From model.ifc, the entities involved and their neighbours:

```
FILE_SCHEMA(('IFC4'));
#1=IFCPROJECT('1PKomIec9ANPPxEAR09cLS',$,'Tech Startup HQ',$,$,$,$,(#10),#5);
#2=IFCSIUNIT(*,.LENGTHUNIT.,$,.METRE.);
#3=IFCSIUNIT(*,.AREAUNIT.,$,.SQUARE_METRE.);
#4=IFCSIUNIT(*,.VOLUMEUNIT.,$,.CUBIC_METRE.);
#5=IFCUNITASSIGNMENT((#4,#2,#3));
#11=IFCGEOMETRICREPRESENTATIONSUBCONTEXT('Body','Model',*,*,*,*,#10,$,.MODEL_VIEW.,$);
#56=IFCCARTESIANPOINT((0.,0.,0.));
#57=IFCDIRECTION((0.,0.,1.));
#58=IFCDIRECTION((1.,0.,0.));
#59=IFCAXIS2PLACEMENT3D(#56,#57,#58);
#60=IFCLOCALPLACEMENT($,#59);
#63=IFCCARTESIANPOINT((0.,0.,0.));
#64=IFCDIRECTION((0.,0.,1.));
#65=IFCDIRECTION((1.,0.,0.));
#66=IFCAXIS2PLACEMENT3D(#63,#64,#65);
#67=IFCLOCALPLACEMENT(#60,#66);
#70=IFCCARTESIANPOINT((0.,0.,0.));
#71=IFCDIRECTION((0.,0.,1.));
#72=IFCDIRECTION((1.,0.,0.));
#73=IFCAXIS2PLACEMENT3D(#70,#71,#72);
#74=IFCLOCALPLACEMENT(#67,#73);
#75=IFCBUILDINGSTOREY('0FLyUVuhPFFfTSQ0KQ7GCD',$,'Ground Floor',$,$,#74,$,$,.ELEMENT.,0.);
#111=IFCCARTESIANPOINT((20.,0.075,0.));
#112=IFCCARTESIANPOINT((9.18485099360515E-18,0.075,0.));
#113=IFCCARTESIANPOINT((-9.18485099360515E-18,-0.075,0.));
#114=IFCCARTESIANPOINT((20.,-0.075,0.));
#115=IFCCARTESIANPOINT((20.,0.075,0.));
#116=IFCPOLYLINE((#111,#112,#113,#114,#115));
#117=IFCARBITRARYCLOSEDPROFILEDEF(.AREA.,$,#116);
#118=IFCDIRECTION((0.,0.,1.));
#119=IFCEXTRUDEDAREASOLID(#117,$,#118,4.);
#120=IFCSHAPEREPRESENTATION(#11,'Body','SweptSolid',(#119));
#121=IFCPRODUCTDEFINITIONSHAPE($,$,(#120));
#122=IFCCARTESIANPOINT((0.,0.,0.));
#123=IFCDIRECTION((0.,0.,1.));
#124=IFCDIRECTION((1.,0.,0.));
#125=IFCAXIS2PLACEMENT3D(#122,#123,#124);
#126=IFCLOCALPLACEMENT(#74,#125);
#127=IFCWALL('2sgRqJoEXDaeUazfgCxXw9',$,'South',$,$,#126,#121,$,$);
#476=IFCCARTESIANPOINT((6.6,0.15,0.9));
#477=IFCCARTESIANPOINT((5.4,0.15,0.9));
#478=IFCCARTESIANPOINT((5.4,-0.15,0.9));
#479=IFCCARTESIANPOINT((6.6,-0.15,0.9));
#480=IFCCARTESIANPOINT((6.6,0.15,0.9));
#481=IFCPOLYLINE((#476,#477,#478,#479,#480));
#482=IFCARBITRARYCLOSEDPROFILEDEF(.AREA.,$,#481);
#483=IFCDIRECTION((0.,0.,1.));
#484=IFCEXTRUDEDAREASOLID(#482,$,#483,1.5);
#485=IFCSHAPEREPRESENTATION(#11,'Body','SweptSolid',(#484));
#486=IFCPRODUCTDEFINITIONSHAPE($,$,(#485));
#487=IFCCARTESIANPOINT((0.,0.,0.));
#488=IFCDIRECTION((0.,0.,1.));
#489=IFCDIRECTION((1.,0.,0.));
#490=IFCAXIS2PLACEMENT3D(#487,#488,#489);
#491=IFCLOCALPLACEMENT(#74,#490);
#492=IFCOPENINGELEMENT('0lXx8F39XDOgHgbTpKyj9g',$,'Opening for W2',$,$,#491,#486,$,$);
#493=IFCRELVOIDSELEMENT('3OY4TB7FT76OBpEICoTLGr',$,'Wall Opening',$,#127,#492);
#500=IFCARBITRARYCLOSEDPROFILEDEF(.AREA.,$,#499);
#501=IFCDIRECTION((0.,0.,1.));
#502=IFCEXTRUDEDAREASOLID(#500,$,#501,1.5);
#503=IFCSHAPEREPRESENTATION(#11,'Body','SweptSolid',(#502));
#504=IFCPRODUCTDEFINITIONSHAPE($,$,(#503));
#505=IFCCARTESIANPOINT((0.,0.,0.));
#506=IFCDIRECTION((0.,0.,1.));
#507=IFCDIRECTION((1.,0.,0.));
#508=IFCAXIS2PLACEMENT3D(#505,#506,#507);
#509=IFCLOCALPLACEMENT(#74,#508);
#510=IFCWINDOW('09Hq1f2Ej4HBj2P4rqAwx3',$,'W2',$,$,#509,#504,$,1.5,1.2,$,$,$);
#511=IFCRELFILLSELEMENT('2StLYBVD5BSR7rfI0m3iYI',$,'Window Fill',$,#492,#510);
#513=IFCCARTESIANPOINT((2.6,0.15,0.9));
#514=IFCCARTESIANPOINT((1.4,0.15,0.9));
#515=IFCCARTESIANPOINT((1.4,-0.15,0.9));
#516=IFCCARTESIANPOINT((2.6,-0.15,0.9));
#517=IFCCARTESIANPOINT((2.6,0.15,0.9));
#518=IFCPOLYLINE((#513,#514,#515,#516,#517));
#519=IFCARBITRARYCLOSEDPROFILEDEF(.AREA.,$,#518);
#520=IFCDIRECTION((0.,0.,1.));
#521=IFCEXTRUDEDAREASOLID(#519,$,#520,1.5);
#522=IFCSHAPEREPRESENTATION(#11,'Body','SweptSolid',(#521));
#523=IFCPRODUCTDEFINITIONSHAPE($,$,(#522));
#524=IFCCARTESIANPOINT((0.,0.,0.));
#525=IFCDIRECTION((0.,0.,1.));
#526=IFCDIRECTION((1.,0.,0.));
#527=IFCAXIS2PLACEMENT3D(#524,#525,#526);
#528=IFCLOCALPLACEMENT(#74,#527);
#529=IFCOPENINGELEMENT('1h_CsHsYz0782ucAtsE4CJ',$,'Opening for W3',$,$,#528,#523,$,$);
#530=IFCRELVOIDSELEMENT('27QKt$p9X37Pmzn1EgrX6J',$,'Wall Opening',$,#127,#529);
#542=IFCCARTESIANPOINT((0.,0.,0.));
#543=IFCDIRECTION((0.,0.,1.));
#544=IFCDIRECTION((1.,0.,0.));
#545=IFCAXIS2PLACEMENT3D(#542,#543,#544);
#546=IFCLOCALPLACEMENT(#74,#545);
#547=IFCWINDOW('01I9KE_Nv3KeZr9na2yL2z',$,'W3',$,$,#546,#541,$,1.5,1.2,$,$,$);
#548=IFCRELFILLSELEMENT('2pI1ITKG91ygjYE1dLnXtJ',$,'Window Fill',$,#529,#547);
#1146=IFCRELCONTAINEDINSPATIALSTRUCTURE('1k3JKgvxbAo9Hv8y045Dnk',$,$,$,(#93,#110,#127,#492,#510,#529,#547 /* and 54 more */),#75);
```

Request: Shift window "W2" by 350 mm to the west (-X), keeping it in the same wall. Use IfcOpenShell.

```python
import ifcopenshell
import ifcopenshell.api.geometry
import ifcopenshell.util.placement
import ifcopenshell.util.unit

model = ifcopenshell.open("model.ifc")
unit_scale = ifcopenshell.util.unit.calculate_unit_scale(model)

window = model.by_guid("09Hq1f2Ej4HBj2P4rqAwx3")
opening = window.FillsVoids[0].RelatingOpeningElement
wall = opening.VoidsElements[0].RelatingBuildingElement

wall_matrix = ifcopenshell.util.placement.get_local_placement(wall.ObjectPlacement)
shift = wall_matrix[:3, 0] * -0.35 / unit_scale
before = ifcopenshell.util.placement.get_local_placement(window.ObjectPlacement)[:3, 3].copy()

# The window is not placed relative to its opening, so move both.
for product in (opening, window):
    matrix = ifcopenshell.util.placement.get_local_placement(product.ObjectPlacement)
    matrix[:3, 3] += shift
    ifcopenshell.api.geometry.edit_object_placement(model, product=product, matrix=matrix, is_si=False)

after = ifcopenshell.util.placement.get_local_placement(window.ObjectPlacement)[:3, 3]
print("window moved by", (after - before).round(3) + 0.0)

model.write("model-out.ifc")
```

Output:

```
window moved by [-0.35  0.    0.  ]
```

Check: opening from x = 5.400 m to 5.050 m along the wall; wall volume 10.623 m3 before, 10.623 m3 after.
